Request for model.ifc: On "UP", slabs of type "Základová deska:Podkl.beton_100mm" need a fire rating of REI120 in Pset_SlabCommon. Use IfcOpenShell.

First a look at what the model holds.

```python
import ifcopenshell
import ifcopenshell.util.element

model = ifcopenshell.open("model.ifc")
print(model.schema)
storey = next(s for s in model.by_type("IfcBuildingStorey") if s.Name == "UP")
slabs = [e for e in ifcopenshell.util.element.get_decomposition(storey) if e.is_a("IfcSlab")]
seen = {}
for e in slabs:
    element_type = ifcopenshell.util.element.get_type(e)
    key = (element_type.Name if element_type != e and element_type else None, ifcopenshell.util.element.get_pset(e, "Pset_SlabCommon", "FireRating"))
    seen[key] = seen.get(key, 0) + 1
for (name, value), count in sorted(seen.items(), key=str):
    print(count, "x", name, "|", value)
```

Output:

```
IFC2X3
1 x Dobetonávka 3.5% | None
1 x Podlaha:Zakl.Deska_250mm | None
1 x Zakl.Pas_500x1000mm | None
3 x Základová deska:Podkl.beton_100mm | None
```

```python
import ifcopenshell
import ifcopenshell.api.pset
import ifcopenshell.util.element

model = ifcopenshell.open("model.ifc")

storey = next(s for s in model.by_type("IfcBuildingStorey") if s.Name == "UP")
slabs = [e for e in ifcopenshell.util.element.get_decomposition(storey) if e.is_a("IfcSlab")]

count = 0
for e in slabs:
    element_type = ifcopenshell.util.element.get_type(e)
    if element_type in (None, e) or element_type.Name != "Základová deska:Podkl.beton_100mm":
        continue
    # add_pset returns the element's existing set when there is one.
    pset = ifcopenshell.api.pset.add_pset(model, product=e, name="Pset_SlabCommon")
    ifcopenshell.api.pset.edit_pset(model, pset=pset, properties={"FireRating": "REI120"})
    count += 1

print(count, "slabs updated")

model.write("model_edited.ifc")
```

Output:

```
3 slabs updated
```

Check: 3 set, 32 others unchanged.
